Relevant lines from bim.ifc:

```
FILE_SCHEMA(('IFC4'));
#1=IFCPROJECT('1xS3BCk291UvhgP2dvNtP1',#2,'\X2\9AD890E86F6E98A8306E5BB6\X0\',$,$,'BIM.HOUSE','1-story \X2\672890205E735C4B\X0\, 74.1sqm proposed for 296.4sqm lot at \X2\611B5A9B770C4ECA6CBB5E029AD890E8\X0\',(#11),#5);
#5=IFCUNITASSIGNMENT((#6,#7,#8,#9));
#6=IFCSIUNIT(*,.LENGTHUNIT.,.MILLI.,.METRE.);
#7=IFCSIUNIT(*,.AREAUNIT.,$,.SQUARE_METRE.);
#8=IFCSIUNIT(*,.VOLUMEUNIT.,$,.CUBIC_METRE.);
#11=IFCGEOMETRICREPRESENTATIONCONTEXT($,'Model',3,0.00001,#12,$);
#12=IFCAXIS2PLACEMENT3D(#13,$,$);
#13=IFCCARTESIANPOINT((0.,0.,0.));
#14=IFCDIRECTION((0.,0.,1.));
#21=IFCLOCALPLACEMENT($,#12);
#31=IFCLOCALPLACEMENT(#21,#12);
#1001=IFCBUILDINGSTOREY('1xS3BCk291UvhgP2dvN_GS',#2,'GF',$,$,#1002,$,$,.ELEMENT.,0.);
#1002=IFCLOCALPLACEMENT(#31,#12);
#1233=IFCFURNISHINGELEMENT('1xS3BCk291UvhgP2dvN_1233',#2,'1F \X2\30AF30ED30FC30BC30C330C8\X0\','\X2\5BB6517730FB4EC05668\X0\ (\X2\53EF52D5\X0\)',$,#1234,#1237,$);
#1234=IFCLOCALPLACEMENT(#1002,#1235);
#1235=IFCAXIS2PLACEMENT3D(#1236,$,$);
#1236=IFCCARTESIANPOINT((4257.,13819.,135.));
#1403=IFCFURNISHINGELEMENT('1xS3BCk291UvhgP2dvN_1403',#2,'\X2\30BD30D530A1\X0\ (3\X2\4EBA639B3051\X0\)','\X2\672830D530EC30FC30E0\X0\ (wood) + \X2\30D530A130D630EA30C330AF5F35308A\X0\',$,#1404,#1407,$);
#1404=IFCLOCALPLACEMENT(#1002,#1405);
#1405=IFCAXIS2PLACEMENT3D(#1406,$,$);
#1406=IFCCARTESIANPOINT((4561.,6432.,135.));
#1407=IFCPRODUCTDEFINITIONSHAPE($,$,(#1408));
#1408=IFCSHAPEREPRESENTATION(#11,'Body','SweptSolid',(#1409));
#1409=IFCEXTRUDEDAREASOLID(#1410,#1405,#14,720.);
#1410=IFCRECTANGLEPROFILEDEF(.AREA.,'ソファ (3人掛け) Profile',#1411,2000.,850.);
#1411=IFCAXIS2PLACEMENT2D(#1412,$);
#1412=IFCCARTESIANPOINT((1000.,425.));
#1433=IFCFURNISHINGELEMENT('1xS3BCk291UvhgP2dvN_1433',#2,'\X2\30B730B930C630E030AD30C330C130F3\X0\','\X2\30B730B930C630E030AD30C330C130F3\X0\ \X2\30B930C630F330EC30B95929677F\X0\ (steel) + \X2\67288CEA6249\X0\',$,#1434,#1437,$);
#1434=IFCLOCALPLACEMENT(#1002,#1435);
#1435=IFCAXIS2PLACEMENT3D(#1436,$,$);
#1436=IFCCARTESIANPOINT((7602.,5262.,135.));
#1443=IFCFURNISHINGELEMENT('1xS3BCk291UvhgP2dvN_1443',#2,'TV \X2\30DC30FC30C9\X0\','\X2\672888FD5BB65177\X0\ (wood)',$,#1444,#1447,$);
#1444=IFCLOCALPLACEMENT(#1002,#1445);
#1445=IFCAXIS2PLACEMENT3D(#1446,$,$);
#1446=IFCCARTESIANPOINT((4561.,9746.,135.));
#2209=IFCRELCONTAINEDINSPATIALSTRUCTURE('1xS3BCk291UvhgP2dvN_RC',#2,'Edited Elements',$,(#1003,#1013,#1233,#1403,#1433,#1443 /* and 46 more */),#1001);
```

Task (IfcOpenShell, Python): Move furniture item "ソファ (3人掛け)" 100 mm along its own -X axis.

```python
import ifcopenshell
import ifcopenshell.api.geometry
import ifcopenshell.util.placement

model = ifcopenshell.open("bim.ifc")

item = model.by_guid("1xS3BCk291UvhgP2dvN_1403")
matrix = ifcopenshell.util.placement.get_local_placement(item.ObjectPlacement)
matrix[:3, 3] -= matrix[:3, 0] * 100.0
ifcopenshell.api.geometry.edit_object_placement(model, product=item, matrix=matrix, is_si=False)

print(ifcopenshell.util.placement.get_local_placement(item.ObjectPlacement).round(3) + 0.0)

model.write("bim_edited.ifc")
```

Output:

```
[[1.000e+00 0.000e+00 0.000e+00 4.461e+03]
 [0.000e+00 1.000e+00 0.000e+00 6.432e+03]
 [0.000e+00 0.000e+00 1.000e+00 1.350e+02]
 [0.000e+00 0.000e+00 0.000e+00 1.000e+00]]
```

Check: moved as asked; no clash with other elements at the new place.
